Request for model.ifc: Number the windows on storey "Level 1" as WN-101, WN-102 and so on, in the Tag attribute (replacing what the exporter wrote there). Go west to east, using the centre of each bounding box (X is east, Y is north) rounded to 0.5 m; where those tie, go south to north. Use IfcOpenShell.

First a look at what the model holds.

```python
import ifcopenshell
import ifcopenshell.util.element
import ifcopenshell.util.placement

model = ifcopenshell.open("model.ifc")
print(model.schema)
storey = next(s for s in model.by_type("IfcBuildingStorey") if s.Name == "Level 1")
windows = [e for e in ifcopenshell.util.element.get_decomposition(storey) if e.is_a("IfcWindow")]
for e in sorted(windows, key=lambda e: e.id()):
    origin = ifcopenshell.util.placement.get_local_placement(e.ObjectPlacement)[:3, 3]
    print(e.id(), e.Tag, e.Name, origin.round(2) + 0.0, sep=" | ")
```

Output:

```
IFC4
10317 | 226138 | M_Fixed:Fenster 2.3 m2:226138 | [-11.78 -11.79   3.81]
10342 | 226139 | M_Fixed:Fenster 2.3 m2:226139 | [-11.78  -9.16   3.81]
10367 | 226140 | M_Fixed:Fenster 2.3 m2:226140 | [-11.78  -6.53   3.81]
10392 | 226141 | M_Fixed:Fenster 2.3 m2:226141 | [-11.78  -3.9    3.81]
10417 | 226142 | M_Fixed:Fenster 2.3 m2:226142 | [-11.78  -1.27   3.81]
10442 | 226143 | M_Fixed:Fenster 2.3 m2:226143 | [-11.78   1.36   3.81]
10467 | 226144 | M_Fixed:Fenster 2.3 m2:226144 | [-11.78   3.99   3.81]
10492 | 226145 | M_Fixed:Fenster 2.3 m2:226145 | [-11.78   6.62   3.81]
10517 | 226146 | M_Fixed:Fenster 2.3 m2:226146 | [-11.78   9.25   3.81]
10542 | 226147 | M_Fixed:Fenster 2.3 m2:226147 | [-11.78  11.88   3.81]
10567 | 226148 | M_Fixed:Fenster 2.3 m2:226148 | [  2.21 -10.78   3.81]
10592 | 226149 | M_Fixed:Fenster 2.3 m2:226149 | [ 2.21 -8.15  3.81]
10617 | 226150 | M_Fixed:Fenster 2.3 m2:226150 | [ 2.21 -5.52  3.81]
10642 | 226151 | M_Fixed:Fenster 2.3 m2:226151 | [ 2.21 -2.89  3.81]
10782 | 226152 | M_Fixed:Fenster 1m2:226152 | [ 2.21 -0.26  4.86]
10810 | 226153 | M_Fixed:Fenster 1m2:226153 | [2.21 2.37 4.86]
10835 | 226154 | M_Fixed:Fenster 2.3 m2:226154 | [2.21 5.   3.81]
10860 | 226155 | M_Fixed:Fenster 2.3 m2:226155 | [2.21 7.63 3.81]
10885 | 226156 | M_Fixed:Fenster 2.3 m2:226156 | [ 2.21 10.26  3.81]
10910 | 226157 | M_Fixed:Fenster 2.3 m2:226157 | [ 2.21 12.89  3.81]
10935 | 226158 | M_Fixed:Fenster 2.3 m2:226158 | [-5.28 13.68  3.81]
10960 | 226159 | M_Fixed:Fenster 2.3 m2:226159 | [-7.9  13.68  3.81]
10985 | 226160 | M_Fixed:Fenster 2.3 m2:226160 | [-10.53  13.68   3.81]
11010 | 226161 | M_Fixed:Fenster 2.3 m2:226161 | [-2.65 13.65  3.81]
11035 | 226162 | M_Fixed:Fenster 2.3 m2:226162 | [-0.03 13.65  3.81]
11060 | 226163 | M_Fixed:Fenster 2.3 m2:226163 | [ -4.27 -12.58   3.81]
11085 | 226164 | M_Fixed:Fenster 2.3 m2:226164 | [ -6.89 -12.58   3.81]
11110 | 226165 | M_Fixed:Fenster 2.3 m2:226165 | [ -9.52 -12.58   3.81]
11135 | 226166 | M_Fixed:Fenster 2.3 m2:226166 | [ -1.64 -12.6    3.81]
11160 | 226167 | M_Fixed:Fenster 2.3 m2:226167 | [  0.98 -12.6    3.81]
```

```python
import ifcopenshell
import ifcopenshell.geom
import ifcopenshell.util.element
import ifcopenshell.util.shape

model = ifcopenshell.open("model.ifc")
settings = ifcopenshell.geom.settings()
settings.set("use-world-coords", True)


def centre(element):
    shape = ifcopenshell.geom.create_shape(settings, element)
    return ifcopenshell.util.shape.get_bbox_centroid(shape.geometry)


storey = next(s for s in model.by_type("IfcBuildingStorey") if s.Name == "Level 1")
windows = [e for e in ifcopenshell.util.element.get_decomposition(storey) if e.is_a("IfcWindow")]

# Insertion points can sit at a corner or the storey origin, so sort by the geometry (in metres).
centres = {e: centre(e) for e in windows}
windows.sort(key=lambda e: (round(centres[e][0] / 0.5), centres[e][1]))

for i, e in enumerate(windows, start=1):
    number = f"WN-1{i:02d}"
    e.Tag = number
    print(e.id(), number)

model.write("model-out.ifc")
```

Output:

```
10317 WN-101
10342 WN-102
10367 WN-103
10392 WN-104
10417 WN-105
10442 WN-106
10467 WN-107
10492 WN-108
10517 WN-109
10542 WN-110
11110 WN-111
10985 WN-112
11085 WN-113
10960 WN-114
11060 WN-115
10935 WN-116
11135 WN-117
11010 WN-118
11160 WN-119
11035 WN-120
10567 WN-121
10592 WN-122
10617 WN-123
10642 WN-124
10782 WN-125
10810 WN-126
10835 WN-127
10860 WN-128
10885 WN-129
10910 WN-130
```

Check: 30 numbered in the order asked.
